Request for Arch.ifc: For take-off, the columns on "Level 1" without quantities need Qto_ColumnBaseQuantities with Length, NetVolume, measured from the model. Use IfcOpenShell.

First a look at what the model holds.

```python
import ifcopenshell
import ifcopenshell.util.element
import ifcopenshell.util.unit

model = ifcopenshell.open("Arch.ifc")
print(model.schema)
for unit_type in ("LENGTHUNIT", "AREAUNIT", "VOLUMEUNIT"):
    print(unit_type, ifcopenshell.util.unit.calculate_unit_scale(model, unit_type))
storey = next(s for s in model.by_type("IfcBuildingStorey") if s.Name == "Level 1")
columns = [e for e in ifcopenshell.util.element.get_decomposition(storey) if e.is_a("IfcColumn")]
for e in sorted(columns, key=lambda e: e.id()):
    print(e.id(), e.is_a(), e.Name, list(ifcopenshell.util.element.get_psets(e, qtos_only=True)), sep=" | ")
```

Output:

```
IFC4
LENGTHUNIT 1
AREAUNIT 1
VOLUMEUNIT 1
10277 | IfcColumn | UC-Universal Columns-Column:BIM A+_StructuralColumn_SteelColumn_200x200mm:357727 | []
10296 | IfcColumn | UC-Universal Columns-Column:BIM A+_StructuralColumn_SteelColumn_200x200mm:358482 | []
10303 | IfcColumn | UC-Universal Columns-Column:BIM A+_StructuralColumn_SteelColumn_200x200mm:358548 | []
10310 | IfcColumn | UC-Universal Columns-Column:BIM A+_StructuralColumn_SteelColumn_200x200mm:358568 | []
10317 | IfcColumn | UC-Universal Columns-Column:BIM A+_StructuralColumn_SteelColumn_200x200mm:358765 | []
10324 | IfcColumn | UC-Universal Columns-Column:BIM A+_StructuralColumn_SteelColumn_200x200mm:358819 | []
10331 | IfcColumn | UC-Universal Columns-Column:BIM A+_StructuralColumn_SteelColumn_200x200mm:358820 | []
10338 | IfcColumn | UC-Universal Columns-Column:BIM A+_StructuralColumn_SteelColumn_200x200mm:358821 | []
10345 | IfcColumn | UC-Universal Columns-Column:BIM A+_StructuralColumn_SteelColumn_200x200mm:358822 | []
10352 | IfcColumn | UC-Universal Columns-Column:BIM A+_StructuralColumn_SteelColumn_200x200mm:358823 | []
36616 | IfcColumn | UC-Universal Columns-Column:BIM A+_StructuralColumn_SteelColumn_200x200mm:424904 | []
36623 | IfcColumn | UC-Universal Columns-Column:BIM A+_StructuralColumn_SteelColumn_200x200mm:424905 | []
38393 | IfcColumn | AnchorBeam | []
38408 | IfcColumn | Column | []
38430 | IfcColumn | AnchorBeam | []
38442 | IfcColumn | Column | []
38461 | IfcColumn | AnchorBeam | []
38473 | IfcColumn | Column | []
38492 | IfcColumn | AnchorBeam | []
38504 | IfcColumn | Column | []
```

```python
import ifcopenshell
import ifcopenshell.api.pset
import ifcopenshell.geom
import ifcopenshell.util.element
import ifcopenshell.util.shape
import ifcopenshell.util.unit

model = ifcopenshell.open("Arch.ifc")
unit_scale = ifcopenshell.util.unit.calculate_unit_scale(model)
volume_scale = ifcopenshell.util.unit.calculate_unit_scale(model, "VOLUMEUNIT")
settings = ifcopenshell.geom.settings()

storey = next(s for s in model.by_type("IfcBuildingStorey") if s.Name == "Level 1")
columns = [e for e in ifcopenshell.util.element.get_decomposition(storey) if e.is_a("IfcColumn")]

for e in sorted(columns, key=lambda e: e.id()):
    if ifcopenshell.util.element.get_psets(e, qtos_only=True, should_inherit=False):
        continue
    # Geometry comes back in metres, in the element's own axes.
    shape = ifcopenshell.geom.create_shape(settings, e)
    values = {
        "Length": ifcopenshell.util.shape.get_z(shape.geometry) / unit_scale,
        "NetVolume": ifcopenshell.util.shape.get_volume(shape.geometry) / volume_scale,
    }
    qto = ifcopenshell.api.pset.add_qto(model, product=e, name="Qto_ColumnBaseQuantities")
    ifcopenshell.api.pset.edit_qto(model, qto=qto, properties=values)
    print(e.id(), {k: round(v, 3) for k, v in values.items()})

model.write("Arch_updated.ifc")
```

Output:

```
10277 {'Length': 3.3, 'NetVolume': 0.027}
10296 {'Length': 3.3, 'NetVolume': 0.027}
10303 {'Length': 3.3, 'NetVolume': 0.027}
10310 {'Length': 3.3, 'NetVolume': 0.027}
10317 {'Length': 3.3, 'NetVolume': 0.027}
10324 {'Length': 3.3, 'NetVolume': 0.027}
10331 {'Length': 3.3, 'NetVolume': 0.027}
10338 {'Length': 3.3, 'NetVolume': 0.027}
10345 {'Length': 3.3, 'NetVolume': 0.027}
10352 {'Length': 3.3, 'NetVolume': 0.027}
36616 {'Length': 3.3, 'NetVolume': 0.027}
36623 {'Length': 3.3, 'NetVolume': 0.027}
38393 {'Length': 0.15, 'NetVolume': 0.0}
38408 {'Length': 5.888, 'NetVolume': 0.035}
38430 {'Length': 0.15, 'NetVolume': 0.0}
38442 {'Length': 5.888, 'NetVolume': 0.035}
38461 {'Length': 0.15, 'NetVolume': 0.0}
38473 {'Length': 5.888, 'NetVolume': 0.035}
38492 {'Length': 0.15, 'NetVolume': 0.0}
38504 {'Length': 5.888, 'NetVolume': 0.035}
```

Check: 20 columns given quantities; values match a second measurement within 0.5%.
